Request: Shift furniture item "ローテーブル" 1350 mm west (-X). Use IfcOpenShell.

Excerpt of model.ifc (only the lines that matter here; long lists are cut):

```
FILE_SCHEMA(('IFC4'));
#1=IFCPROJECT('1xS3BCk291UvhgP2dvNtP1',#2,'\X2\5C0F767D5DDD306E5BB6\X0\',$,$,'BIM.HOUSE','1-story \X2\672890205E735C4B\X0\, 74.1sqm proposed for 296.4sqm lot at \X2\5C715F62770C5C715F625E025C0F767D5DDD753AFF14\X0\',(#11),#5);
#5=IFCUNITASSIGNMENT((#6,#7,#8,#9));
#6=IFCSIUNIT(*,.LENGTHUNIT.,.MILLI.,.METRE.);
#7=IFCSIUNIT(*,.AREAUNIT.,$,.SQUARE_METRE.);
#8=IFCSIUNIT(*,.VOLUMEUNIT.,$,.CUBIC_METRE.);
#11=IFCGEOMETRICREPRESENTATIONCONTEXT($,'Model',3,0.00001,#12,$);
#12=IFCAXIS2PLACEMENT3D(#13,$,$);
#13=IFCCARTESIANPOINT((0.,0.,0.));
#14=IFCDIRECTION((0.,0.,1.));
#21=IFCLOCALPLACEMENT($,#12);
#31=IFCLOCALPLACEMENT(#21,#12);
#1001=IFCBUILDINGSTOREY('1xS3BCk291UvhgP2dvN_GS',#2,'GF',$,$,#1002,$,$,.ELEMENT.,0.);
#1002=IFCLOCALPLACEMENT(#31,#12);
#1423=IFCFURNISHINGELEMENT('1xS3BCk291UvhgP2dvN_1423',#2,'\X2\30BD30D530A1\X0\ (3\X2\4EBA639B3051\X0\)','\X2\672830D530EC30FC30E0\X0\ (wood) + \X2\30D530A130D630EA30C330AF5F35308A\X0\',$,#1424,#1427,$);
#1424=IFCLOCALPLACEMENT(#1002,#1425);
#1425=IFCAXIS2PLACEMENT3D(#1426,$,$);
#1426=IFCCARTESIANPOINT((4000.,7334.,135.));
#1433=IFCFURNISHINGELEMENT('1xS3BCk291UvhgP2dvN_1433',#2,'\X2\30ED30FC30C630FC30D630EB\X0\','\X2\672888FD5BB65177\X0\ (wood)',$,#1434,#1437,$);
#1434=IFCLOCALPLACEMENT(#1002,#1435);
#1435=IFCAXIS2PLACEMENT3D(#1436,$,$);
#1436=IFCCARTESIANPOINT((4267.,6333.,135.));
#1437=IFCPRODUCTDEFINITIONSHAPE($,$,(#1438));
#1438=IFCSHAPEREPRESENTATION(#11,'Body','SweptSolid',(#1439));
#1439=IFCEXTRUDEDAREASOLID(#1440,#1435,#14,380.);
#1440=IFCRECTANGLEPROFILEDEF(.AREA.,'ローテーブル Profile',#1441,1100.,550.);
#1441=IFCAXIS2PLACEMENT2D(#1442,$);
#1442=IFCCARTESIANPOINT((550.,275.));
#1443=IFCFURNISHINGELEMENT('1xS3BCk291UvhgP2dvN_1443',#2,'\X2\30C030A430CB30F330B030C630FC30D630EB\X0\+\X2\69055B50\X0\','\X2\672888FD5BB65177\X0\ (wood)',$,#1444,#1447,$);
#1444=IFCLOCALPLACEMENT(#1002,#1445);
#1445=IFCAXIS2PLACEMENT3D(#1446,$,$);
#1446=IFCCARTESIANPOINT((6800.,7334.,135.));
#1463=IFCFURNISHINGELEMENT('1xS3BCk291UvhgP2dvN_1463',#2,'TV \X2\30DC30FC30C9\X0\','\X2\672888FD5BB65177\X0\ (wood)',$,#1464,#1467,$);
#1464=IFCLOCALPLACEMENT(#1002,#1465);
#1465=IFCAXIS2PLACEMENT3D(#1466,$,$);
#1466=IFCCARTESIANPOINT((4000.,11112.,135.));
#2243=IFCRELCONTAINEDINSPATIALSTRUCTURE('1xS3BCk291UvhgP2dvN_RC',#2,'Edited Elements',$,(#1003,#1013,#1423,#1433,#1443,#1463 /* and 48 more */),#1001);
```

```python
import ifcopenshell
import ifcopenshell.api.geometry
import ifcopenshell.util.placement
import ifcopenshell.util.unit

model = ifcopenshell.open("model.ifc")
unit_scale = ifcopenshell.util.unit.calculate_unit_scale(model)

item = model.by_guid("1xS3BCk291UvhgP2dvN_1433")
matrix = ifcopenshell.util.placement.get_local_placement(item.ObjectPlacement)
matrix[0, 3] -= 1.35 / unit_scale
ifcopenshell.api.geometry.edit_object_placement(model, product=item, matrix=matrix, is_si=False)

print(ifcopenshell.util.placement.get_local_placement(item.ObjectPlacement).round(3) + 0.0)

model.write("model-out.ifc")
```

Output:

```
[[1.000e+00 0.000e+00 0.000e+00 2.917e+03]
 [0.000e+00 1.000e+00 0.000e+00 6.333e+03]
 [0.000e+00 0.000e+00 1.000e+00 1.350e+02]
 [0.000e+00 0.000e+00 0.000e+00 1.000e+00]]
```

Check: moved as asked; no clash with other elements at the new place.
